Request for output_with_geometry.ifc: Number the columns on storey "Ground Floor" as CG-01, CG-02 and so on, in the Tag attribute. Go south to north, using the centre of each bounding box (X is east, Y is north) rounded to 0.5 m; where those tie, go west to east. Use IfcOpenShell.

First a look at what the model holds.

```python
import ifcopenshell
import ifcopenshell.util.element
import ifcopenshell.util.placement

model = ifcopenshell.open("output_with_geometry.ifc")
print(model.schema)
storey = next(s for s in model.by_type("IfcBuildingStorey") if s.Name == "Ground Floor")
columns = [e for e in ifcopenshell.util.element.get_decomposition(storey) if e.is_a("IfcColumn")]
for e in sorted(columns, key=lambda e: e.id()):
    origin = ifcopenshell.util.placement.get_local_placement(e.ObjectPlacement)[:3, 3]
    print(e.id(), e.Tag, e.Name, origin.round(2) + 0.0, sep=" | ")
```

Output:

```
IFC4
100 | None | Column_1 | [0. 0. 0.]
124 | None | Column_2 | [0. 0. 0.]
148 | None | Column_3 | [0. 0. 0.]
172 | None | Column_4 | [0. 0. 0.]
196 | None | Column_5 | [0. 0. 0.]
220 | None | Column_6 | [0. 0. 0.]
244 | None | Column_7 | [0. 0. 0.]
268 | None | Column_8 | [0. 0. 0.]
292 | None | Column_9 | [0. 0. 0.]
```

```python
import ifcopenshell
import ifcopenshell.geom
import ifcopenshell.util.element
import ifcopenshell.util.shape

model = ifcopenshell.open("output_with_geometry.ifc")
settings = ifcopenshell.geom.settings()
settings.set("use-world-coords", True)


def centre(element):
    shape = ifcopenshell.geom.create_shape(settings, element)
    return ifcopenshell.util.shape.get_bbox_centroid(shape.geometry)


storey = next(s for s in model.by_type("IfcBuildingStorey") if s.Name == "Ground Floor")
columns = [e for e in ifcopenshell.util.element.get_decomposition(storey) if e.is_a("IfcColumn")]

# Insertion points can sit at a corner or the storey origin, so sort by the geometry (in metres).
centres = {e: centre(e) for e in columns}
columns.sort(key=lambda e: (round(centres[e][1] / 0.5), centres[e][0]))

for i, e in enumerate(columns, start=1):
    number = f"CG-{i:02d}"
    e.Tag = number
    print(e.id(), number)

model.write("output_with_geometry_v2.ifc")
```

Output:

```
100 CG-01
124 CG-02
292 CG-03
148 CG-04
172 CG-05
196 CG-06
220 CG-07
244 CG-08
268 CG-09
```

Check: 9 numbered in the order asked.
